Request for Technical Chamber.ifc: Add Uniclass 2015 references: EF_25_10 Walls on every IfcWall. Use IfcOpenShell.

First a look at what the model holds.

```python
import ifcopenshell

model = ifcopenshell.open("Technical Chamber.ifc")
print(model.schema)
print("classifications:", [c.Name for c in model.by_type("IfcClassification")])
for ifc_class in ("IfcDoor", "IfcRoof", "IfcStair", "IfcWall", "IfcWindow"):
    print(ifc_class, len(model.by_type(ifc_class)))
```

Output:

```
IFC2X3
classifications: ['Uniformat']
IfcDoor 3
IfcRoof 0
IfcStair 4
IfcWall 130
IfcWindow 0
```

```python
import ifcopenshell
import ifcopenshell.api.classification

model = ifcopenshell.open("Technical Chamber.ifc")

# IFC2X3 requires Source and Edition and has no link from the project to the system.
system = model.create_entity("IfcClassification", Source="NBS", Edition="2015", Name="Uniclass 2015")

codes = {
    "IfcWall": ("EF_25_10", "Walls"),
}
for ifc_class, (code, name) in codes.items():
    products = model.by_type(ifc_class)
    ifcopenshell.api.classification.add_reference(
        model, products=products, classification=system, identification=code, name=name
    )
    print(code, len(products))

model.write("Technical Chamber_edited.ifc")
```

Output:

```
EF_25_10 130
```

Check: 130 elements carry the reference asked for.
